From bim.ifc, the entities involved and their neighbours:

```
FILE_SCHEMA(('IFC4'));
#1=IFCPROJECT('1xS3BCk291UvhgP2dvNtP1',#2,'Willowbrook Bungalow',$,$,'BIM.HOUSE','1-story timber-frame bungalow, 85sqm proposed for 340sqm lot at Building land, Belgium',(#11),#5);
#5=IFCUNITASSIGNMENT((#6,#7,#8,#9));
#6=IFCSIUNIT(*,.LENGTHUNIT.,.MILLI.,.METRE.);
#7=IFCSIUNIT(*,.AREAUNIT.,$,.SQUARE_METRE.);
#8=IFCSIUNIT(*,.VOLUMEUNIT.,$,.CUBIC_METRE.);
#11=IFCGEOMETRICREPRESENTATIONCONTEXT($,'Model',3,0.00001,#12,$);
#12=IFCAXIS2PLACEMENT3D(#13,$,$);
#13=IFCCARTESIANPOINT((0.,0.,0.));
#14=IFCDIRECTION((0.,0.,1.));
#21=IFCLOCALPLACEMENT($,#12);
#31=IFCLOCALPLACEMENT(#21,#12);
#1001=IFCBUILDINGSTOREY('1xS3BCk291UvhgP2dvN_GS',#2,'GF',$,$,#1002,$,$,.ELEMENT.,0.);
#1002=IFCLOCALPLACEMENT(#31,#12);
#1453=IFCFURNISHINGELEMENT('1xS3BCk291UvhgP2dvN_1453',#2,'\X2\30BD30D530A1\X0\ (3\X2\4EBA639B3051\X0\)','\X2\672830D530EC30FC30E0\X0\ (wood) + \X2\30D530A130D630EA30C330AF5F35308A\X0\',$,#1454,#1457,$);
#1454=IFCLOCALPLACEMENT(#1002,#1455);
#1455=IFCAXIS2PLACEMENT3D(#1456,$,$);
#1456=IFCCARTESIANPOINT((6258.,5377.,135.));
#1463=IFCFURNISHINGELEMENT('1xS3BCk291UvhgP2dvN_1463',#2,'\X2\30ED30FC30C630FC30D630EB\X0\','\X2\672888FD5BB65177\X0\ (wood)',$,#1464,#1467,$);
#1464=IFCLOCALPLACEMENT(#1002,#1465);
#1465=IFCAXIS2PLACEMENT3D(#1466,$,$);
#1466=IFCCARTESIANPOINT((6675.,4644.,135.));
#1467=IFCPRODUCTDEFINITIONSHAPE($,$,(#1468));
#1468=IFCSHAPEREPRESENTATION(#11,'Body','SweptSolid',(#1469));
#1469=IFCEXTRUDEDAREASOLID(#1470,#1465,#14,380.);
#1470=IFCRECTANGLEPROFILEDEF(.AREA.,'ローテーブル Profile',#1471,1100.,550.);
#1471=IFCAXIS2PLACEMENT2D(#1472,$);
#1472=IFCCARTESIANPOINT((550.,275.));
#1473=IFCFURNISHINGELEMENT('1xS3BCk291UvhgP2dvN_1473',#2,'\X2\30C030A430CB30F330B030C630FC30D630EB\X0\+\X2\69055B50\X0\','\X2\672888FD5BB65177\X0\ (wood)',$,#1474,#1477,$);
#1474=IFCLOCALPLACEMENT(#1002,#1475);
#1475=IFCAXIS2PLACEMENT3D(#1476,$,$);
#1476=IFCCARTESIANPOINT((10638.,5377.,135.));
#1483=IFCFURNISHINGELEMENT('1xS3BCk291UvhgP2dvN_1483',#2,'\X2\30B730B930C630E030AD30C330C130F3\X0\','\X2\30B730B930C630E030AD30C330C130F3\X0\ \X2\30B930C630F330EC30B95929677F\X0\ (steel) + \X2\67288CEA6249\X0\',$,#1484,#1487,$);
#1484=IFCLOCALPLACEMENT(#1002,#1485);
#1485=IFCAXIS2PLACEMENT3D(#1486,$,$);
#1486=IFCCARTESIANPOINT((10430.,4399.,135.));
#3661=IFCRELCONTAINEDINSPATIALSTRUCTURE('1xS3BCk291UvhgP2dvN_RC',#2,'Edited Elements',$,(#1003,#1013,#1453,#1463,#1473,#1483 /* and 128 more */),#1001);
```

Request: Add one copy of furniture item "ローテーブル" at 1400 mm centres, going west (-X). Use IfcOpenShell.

```python
import numpy as np
import ifcopenshell
import ifcopenshell.api.geometry
import ifcopenshell.api.root
import ifcopenshell.util.element
import ifcopenshell.util.placement
import ifcopenshell.util.unit

model = ifcopenshell.open("bim.ifc")
unit_scale = ifcopenshell.util.unit.calculate_unit_scale(model)


def reuse_history(source, copy):
    """copy_class also copies each property set's owner history, people and application; keep the originals."""
    for rel in copy.IsDefinedBy:
        if rel.is_a("IfcRelDefinesByProperties") and (history := rel.RelatingPropertyDefinition.OwnerHistory):
            rel.RelatingPropertyDefinition.OwnerHistory = source.OwnerHistory
            ifcopenshell.util.element.remove_deep2(model, history)


source = model.by_guid("1xS3BCk291UvhgP2dvN_1463")
base = ifcopenshell.util.placement.get_local_placement(source.ObjectPlacement)
step = np.array([-1.0, 0.0, 0.0]) * 1.4 / unit_scale

for i in range(1, 2):
    copy = ifcopenshell.api.root.copy_class(model, product=source)
    copy.Representation = ifcopenshell.util.element.copy_deep(
        model, source.Representation, exclude=["IfcGeometricRepresentationContext", "IfcRepresentationMap"]
    )
    reuse_history(source, copy)
    matrix = base.copy()
    matrix[:3, 3] += i * step
    print("added at", matrix[:3, 3].round(3) + 0.0)
    ifcopenshell.api.geometry.edit_object_placement(model, product=copy, matrix=matrix, is_si=False)

model.write("bim_edited.ifc")
```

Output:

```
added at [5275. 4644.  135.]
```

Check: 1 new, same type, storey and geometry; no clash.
